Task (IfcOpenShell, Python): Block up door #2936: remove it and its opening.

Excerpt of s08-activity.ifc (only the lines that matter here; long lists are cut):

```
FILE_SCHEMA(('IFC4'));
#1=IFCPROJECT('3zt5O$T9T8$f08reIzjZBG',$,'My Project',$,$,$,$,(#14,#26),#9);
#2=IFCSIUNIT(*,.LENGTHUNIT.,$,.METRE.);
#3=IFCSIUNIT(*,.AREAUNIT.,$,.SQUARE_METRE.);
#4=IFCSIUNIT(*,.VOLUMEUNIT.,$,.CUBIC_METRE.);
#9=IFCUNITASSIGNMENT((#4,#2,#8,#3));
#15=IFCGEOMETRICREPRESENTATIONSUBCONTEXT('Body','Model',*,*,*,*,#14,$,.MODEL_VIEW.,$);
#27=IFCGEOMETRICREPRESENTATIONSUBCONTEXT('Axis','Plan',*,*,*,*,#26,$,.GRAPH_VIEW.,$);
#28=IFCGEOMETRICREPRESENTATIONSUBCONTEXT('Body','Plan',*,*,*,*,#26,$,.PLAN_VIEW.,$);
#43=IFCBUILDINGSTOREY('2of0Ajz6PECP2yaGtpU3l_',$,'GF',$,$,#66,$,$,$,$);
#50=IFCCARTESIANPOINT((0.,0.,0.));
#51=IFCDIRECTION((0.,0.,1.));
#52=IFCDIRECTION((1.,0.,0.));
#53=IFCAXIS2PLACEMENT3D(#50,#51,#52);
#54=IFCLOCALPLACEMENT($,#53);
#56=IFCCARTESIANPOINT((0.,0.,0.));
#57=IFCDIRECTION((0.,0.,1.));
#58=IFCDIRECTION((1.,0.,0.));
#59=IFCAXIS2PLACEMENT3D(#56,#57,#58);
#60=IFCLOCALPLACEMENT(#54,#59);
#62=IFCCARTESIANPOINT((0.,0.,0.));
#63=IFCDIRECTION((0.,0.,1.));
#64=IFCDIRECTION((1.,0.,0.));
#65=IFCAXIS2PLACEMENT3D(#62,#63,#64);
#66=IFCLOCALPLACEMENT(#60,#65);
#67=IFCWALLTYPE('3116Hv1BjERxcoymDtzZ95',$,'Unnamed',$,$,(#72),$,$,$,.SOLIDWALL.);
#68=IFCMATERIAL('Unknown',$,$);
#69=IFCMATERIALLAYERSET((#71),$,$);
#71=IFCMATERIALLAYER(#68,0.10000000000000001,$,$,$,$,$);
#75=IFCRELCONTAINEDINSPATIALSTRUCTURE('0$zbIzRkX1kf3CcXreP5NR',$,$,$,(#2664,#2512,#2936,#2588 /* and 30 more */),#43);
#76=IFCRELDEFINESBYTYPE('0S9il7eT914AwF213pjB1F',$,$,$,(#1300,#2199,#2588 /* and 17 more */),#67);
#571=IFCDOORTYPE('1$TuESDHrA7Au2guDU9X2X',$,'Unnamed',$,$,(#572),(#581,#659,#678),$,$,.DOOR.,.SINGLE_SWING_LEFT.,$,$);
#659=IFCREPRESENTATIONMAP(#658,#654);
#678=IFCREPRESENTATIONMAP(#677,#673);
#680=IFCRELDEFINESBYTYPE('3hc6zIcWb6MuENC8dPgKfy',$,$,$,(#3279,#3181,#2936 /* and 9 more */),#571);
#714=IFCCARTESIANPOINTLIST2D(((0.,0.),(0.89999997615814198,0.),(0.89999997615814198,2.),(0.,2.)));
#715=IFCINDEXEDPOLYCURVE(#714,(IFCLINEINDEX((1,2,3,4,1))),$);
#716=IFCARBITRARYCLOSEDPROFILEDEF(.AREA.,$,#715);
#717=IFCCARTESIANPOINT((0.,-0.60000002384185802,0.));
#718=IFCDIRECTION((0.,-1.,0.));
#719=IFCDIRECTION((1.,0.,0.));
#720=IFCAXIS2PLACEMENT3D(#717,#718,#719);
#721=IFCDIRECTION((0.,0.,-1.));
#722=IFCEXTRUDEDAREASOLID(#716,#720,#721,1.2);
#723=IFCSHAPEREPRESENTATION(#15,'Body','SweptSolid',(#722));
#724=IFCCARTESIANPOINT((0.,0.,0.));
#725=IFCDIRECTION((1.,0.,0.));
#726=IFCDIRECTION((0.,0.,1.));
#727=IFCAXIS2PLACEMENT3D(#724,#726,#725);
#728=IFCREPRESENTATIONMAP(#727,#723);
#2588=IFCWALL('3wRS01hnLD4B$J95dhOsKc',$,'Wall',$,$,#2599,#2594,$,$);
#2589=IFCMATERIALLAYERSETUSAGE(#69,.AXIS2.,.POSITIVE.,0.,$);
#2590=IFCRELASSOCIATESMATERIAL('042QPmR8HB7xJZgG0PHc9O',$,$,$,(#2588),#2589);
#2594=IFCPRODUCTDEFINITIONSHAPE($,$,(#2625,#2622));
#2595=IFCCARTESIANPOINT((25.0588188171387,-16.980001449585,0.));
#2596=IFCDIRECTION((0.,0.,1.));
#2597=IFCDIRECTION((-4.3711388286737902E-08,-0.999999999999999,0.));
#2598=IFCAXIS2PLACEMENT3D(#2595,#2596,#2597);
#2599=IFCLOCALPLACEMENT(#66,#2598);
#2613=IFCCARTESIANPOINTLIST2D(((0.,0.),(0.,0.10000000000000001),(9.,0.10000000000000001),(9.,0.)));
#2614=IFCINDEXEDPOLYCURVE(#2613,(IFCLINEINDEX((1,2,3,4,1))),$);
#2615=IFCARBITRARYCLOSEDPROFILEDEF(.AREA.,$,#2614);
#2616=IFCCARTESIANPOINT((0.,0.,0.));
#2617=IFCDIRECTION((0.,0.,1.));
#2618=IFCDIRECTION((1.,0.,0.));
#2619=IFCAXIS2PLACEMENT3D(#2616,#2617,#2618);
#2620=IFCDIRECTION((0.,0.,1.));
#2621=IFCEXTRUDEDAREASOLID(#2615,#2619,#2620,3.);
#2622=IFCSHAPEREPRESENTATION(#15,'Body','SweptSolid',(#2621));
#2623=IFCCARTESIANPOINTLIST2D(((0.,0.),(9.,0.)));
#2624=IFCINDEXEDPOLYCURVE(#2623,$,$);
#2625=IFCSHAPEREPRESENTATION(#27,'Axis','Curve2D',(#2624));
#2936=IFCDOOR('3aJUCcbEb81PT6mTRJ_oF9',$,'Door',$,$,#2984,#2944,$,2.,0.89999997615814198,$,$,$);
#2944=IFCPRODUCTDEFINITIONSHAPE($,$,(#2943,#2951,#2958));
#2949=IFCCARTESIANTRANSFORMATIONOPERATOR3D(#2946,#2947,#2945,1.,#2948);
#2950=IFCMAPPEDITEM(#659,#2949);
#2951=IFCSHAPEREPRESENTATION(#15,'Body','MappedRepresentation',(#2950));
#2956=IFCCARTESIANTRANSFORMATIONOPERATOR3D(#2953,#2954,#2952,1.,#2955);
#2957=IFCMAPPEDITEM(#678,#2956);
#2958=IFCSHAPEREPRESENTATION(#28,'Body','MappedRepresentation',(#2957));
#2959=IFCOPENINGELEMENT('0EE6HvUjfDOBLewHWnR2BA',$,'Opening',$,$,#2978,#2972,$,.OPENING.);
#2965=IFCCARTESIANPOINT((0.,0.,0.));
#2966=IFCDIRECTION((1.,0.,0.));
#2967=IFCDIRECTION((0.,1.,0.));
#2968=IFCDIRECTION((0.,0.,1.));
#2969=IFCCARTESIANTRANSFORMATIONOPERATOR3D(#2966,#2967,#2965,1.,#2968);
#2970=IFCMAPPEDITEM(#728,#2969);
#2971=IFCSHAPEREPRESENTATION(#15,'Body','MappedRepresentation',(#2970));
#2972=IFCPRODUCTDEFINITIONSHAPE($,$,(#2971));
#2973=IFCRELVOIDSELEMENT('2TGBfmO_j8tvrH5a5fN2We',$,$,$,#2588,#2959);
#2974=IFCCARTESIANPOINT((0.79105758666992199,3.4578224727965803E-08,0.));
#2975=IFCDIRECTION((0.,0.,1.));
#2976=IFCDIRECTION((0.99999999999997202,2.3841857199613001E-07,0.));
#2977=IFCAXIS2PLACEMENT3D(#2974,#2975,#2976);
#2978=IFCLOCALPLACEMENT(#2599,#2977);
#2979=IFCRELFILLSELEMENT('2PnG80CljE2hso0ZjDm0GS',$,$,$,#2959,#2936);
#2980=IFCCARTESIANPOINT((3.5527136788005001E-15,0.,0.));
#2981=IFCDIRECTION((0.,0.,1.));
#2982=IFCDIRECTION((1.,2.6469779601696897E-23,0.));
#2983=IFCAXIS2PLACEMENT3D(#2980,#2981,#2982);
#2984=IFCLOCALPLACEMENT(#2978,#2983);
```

```python
import ifcopenshell
import ifcopenshell.api.feature
import ifcopenshell.api.root
import ifcopenshell.geom
import ifcopenshell.util.shape

model = ifcopenshell.open("s08-activity.ifc")
settings = ifcopenshell.geom.settings()


def volume(element):
    """Net volume in cubic metres, openings subtracted."""
    shape = ifcopenshell.geom.create_shape(settings, element)
    return ifcopenshell.util.shape.get_volume(shape.geometry)


door = model.by_guid("3aJUCcbEb81PT6mTRJ_oF9")
opening = door.FillsVoids[0].RelatingOpeningElement
wall = opening.VoidsElements[0].RelatingBuildingElement
before = volume(wall)

ifcopenshell.api.root.remove_product(model, product=door)
ifcopenshell.api.feature.remove_feature(model, feature=opening)

after = volume(wall)

print(f"wall volume {before:.3f} -> {after:.3f} m3")

model.write("s08-activity-out.ifc")
```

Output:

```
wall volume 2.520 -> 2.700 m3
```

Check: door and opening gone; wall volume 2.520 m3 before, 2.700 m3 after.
